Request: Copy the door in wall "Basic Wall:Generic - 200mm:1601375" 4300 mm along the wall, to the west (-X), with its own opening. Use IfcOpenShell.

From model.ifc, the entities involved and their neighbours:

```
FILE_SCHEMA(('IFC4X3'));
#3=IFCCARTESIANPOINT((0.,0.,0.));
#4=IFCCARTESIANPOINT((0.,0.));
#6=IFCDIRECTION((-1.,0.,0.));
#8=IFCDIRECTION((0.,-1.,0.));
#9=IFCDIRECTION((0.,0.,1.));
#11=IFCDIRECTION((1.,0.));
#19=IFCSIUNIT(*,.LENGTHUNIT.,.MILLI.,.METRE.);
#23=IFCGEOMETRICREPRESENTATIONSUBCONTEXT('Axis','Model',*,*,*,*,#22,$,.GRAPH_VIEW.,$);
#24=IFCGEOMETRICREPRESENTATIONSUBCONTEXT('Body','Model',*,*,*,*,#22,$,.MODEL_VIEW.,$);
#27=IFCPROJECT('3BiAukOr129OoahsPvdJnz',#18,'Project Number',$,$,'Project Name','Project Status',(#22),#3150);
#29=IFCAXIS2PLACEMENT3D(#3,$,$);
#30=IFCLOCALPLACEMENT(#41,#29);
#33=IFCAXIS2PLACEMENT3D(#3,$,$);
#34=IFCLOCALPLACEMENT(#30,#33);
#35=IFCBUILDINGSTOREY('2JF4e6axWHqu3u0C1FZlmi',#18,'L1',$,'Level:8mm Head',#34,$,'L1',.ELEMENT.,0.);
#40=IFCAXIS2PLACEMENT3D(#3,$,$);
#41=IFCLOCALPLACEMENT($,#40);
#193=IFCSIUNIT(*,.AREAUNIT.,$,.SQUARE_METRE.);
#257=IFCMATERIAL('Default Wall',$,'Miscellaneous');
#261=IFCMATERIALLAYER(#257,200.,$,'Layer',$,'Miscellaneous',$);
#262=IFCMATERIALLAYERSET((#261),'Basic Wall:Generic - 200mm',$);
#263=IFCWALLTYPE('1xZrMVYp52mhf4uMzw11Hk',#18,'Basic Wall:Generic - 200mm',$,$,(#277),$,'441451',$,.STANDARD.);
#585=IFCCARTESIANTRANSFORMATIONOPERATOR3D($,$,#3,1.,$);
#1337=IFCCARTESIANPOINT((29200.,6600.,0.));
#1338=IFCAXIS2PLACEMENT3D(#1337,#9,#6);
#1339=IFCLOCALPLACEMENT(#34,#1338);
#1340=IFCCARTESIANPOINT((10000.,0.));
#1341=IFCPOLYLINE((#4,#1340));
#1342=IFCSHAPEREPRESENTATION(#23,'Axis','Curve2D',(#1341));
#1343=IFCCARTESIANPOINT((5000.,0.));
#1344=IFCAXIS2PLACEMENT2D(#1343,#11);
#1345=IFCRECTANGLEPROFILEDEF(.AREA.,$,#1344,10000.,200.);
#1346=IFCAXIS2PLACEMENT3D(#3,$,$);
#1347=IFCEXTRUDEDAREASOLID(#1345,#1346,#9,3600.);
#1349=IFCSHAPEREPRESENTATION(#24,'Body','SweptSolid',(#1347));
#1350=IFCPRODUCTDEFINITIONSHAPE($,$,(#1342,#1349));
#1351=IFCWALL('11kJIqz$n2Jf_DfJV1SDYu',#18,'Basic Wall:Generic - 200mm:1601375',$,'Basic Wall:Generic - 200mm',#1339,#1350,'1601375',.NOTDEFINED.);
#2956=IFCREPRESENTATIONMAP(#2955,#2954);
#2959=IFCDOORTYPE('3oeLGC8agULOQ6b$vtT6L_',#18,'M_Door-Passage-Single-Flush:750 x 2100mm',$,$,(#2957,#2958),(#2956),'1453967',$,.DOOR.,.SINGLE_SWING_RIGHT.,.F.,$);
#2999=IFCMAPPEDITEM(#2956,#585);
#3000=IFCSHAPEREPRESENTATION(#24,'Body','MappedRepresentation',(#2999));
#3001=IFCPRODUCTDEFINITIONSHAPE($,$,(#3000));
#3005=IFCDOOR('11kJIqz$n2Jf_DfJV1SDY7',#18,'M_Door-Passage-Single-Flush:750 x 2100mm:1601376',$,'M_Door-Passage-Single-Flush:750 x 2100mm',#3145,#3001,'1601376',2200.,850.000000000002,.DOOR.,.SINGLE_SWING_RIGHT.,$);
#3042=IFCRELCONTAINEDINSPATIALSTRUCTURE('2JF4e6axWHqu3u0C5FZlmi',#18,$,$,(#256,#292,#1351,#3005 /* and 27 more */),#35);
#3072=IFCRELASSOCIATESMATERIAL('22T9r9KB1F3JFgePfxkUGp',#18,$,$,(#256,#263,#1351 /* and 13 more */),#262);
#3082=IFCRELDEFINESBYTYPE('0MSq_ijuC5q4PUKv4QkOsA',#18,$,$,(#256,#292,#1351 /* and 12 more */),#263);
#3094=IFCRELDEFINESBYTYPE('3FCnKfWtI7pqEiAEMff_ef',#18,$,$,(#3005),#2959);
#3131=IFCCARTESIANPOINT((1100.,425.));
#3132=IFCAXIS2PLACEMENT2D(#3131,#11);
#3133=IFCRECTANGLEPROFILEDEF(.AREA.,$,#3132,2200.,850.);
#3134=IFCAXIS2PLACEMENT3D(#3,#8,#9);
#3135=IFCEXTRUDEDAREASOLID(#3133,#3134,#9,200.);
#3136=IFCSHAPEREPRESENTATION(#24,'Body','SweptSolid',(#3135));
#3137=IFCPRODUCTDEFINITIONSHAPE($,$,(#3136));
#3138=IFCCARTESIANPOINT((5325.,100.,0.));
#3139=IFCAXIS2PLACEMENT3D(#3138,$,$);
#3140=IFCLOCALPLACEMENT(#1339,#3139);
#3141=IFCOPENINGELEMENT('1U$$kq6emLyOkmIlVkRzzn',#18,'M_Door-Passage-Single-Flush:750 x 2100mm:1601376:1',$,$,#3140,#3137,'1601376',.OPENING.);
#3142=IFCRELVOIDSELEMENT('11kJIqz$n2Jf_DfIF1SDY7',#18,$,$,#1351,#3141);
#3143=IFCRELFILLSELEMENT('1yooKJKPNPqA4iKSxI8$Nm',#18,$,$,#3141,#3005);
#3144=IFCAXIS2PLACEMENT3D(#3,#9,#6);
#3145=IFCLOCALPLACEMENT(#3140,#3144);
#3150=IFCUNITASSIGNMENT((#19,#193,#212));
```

```python
import ifcopenshell
import ifcopenshell.api.feature
import ifcopenshell.api.geometry
import ifcopenshell.api.root
import ifcopenshell.geom
import ifcopenshell.util.element
import ifcopenshell.util.placement
import ifcopenshell.util.shape

model = ifcopenshell.open("model.ifc")
settings = ifcopenshell.geom.settings()


def volume(element):
    """Net volume in cubic metres, openings subtracted."""
    shape = ifcopenshell.geom.create_shape(settings, element)
    return ifcopenshell.util.shape.get_volume(shape.geometry)


def reuse_history(source, copy):
    """copy_class also copies each property set's owner history, people and application; keep the originals."""
    for rel in copy.IsDefinedBy:
        if rel.is_a("IfcRelDefinesByProperties") and (history := rel.RelatingPropertyDefinition.OwnerHistory):
            rel.RelatingPropertyDefinition.OwnerHistory = source.OwnerHistory
            ifcopenshell.util.element.remove_deep2(model, history)


door = model.by_guid("11kJIqz$n2Jf_DfJV1SDY7")
opening = door.FillsVoids[0].RelatingOpeningElement
wall = opening.VoidsElements[0].RelatingBuildingElement
before = volume(wall)
shift = ifcopenshell.util.placement.get_local_placement(wall.ObjectPlacement)[:3, 0] * 4300.0

# copy_class copies the void relationship, type, container and properties, but no geometry.
new_opening = ifcopenshell.api.root.copy_class(model, product=opening)
new_opening.Representation = ifcopenshell.util.element.copy_deep(
    model, opening.Representation, exclude=["IfcGeometricRepresentationContext", "IfcRepresentationMap"]
)
new_opening.Name = "M_Door-Passage-Single-Flush:750 x 2100mm"
new_opening.Tag = None
new_door = ifcopenshell.api.root.copy_class(model, product=door)
new_door.Representation = ifcopenshell.util.element.copy_deep(
    model, door.Representation, exclude=["IfcGeometricRepresentationContext", "IfcRepresentationMap"]
)
new_door.Name = "M_Door-Passage-Single-Flush:750 x 2100mm"
new_door.Tag = None
reuse_history(door, new_door)
ifcopenshell.api.feature.add_filling(model, opening=new_opening, element=new_door)

for old, new in ((opening, new_opening), (door, new_door)):
    matrix = ifcopenshell.util.placement.get_local_placement(old.ObjectPlacement)
    matrix[:3, 3] += shift
    ifcopenshell.api.geometry.edit_object_placement(model, product=new, matrix=matrix, is_si=False)

after = volume(wall)

print(f"wall volume {before:.3f} -> {after:.3f} m3")

model.write("model_edited.ifc")
```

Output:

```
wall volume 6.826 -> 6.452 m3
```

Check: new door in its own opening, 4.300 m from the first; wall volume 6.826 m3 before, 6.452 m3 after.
